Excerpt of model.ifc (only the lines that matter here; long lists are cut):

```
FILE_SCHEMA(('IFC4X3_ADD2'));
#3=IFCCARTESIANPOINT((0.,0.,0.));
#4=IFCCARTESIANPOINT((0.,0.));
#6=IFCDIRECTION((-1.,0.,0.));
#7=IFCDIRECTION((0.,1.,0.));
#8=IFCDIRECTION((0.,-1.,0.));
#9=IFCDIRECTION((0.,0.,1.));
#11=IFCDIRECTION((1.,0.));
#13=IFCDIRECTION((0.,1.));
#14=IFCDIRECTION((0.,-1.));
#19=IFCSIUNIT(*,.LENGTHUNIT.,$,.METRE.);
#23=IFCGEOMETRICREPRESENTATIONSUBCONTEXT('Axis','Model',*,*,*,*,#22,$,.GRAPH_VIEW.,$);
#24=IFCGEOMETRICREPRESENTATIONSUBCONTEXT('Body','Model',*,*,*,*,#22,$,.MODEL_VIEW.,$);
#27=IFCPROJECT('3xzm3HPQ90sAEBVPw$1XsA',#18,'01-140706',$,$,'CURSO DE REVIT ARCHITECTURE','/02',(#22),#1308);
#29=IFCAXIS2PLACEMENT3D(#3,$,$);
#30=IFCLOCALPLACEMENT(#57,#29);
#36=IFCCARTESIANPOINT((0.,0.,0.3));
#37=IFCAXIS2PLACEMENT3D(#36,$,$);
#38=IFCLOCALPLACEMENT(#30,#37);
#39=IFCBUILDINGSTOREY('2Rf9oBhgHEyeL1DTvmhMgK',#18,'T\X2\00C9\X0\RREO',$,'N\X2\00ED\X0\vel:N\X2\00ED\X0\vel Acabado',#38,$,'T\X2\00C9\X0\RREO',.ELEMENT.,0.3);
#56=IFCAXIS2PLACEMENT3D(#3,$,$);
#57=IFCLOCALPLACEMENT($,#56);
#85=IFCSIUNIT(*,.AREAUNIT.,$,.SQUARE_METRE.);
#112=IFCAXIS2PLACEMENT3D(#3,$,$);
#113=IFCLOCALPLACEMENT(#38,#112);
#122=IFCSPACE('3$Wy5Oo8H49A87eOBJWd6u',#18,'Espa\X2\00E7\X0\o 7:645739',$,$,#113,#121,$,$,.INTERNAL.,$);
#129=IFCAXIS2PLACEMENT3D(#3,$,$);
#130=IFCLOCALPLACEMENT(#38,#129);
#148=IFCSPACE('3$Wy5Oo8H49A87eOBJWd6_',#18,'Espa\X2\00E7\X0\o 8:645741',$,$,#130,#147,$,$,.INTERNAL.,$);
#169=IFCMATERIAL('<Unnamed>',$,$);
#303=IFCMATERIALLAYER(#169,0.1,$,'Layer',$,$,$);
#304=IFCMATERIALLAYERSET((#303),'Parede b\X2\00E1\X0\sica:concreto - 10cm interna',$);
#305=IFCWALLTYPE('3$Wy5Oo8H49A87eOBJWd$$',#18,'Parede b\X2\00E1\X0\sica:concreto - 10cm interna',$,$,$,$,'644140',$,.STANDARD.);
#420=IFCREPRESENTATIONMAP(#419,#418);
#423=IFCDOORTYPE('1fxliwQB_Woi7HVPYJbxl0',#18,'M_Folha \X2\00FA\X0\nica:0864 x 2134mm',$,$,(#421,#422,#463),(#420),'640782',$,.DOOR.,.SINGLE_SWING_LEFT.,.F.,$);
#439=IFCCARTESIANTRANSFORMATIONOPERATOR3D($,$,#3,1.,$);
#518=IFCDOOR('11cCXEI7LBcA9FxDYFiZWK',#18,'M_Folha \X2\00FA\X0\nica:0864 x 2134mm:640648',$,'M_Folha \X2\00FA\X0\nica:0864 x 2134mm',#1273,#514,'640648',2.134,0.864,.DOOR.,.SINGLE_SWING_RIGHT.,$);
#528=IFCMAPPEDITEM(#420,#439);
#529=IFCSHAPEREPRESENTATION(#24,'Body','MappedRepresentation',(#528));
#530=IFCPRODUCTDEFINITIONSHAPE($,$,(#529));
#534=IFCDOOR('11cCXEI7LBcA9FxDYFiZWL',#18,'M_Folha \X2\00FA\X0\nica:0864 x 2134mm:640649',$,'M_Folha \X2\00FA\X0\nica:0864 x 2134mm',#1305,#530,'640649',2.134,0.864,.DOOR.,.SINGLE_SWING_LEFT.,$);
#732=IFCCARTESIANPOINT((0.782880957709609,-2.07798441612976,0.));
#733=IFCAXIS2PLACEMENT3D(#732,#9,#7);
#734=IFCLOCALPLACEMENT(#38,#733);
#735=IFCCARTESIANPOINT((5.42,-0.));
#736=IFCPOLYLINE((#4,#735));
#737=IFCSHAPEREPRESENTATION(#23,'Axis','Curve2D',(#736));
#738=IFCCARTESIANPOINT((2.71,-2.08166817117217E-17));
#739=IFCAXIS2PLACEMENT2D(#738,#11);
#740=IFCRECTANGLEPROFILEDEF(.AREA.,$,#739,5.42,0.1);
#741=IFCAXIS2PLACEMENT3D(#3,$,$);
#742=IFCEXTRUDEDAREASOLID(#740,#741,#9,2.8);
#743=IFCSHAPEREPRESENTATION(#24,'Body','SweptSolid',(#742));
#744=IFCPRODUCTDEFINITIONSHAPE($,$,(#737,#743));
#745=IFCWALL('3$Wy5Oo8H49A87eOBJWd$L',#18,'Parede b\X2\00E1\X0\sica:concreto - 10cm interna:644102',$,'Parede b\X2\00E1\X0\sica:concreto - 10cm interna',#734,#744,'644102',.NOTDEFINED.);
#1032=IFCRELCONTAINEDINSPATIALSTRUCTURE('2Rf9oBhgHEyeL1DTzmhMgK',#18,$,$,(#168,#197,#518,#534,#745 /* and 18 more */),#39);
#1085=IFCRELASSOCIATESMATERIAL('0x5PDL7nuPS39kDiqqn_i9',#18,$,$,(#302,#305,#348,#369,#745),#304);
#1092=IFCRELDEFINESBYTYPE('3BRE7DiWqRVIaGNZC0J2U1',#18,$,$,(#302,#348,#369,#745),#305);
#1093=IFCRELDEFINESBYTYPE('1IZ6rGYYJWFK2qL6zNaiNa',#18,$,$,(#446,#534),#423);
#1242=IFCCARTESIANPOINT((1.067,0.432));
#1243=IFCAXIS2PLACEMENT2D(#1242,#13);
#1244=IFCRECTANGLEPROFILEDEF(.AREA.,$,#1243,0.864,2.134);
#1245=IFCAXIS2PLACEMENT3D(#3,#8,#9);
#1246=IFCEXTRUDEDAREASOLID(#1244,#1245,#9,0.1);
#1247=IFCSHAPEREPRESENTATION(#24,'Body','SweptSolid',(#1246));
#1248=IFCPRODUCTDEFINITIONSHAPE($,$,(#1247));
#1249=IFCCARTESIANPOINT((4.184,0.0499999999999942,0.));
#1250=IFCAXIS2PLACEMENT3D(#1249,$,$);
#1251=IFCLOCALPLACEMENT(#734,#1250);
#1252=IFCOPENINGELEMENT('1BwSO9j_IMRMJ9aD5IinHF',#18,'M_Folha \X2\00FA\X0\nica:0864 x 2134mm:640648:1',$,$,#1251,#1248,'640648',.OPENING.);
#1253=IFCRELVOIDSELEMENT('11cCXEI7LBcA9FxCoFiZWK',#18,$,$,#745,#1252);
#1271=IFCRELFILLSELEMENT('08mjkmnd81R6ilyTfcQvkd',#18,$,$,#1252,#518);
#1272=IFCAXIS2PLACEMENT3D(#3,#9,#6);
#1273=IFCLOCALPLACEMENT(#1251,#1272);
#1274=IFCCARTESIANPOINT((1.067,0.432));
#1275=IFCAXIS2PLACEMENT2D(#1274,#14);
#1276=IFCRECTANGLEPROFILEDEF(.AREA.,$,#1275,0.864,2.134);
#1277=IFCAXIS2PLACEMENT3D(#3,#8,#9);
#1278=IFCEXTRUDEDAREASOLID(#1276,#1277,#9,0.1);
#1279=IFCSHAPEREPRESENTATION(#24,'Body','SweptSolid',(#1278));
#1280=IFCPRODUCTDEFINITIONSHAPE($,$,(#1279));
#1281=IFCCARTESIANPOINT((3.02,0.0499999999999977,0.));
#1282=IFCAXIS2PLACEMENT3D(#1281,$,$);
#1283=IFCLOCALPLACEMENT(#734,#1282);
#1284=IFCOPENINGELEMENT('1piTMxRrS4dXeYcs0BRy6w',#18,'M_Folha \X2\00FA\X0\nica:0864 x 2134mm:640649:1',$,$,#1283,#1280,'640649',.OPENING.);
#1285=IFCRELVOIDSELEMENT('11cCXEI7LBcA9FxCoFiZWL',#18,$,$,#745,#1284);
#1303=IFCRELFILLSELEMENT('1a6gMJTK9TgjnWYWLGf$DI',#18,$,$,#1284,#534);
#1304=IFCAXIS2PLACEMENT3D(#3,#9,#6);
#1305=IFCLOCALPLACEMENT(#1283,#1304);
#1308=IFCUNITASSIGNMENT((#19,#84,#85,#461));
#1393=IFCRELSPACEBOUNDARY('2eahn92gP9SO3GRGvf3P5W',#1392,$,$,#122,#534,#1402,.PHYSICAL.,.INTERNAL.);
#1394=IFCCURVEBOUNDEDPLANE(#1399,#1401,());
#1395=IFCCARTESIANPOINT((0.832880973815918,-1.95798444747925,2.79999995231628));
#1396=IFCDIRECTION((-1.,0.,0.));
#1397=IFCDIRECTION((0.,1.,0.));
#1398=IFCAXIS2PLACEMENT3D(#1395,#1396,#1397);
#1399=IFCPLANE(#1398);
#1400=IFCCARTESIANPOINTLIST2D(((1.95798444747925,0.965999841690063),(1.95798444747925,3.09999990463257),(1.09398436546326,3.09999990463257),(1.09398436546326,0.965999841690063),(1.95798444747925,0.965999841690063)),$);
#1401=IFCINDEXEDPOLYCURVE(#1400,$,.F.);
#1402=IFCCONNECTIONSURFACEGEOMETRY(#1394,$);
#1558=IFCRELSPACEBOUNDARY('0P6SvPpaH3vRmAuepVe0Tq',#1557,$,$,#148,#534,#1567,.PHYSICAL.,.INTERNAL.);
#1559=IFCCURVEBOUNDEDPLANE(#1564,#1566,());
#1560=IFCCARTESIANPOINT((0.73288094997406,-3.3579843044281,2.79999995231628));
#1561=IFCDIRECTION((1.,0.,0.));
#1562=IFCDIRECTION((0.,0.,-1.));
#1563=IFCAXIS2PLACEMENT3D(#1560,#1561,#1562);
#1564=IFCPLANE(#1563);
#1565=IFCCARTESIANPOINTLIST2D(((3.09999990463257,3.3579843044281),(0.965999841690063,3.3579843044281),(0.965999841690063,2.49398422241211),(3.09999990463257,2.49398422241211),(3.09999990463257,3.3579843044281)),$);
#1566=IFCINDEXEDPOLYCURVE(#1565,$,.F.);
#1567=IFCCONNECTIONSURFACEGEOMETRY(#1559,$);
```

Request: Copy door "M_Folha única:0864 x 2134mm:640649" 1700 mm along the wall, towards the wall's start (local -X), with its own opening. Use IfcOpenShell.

```python
import numpy as np
import ifcopenshell
import ifcopenshell.api.feature
import ifcopenshell.api.geometry
import ifcopenshell.api.root
import ifcopenshell.geom
import ifcopenshell.util.element
import ifcopenshell.util.placement
import ifcopenshell.util.shape
import ifcopenshell.util.unit

model = ifcopenshell.open("model.ifc")
unit_scale = ifcopenshell.util.unit.calculate_unit_scale(model)
settings = ifcopenshell.geom.settings()


def volume(element):
    """Net volume in cubic metres, openings subtracted."""
    shape = ifcopenshell.geom.create_shape(settings, element)
    return ifcopenshell.util.shape.get_volume(shape.geometry)


def reuse_history(source, copy):
    """copy_class also copies each property set's owner history, people and application; keep the originals."""
    for rel in copy.IsDefinedBy:
        if rel.is_a("IfcRelDefinesByProperties") and (history := rel.RelatingPropertyDefinition.OwnerHistory):
            rel.RelatingPropertyDefinition.OwnerHistory = source.OwnerHistory
            ifcopenshell.util.element.remove_deep2(model, history)


door = model.by_guid("11cCXEI7LBcA9FxDYFiZWL")
opening = door.FillsVoids[0].RelatingOpeningElement
wall = opening.VoidsElements[0].RelatingBuildingElement
before = volume(wall)
shift = ifcopenshell.util.placement.get_local_placement(wall.ObjectPlacement)[:3, 0] * -1.7 / unit_scale

# copy_class copies the void relationship, type, container and properties, but no geometry.
new_opening = ifcopenshell.api.root.copy_class(model, product=opening)
new_opening.Representation = ifcopenshell.util.element.copy_deep(
    model, opening.Representation, exclude=["IfcGeometricRepresentationContext", "IfcRepresentationMap"]
)
new_opening.Name = "M_Folha única:0864 x 2134mm"
new_opening.Tag = None
new_door = ifcopenshell.api.root.copy_class(model, product=door)
new_door.Representation = ifcopenshell.util.element.copy_deep(
    model, door.Representation, exclude=["IfcGeometricRepresentationContext", "IfcRepresentationMap"]
)
new_door.Name = "M_Folha única:0864 x 2134mm"
new_door.Tag = None
reuse_history(door, new_door)
ifcopenshell.api.feature.add_filling(model, opening=new_opening, element=new_door)

for old, new in ((opening, new_opening), (door, new_door)):
    matrix = ifcopenshell.util.placement.get_local_placement(old.ObjectPlacement)
    matrix[:3, 3] += shift
    ifcopenshell.api.geometry.edit_object_placement(model, product=new, matrix=matrix, is_si=False)

# The copied space boundaries still share their surfaces with the original.
for rel in new_door.ProvidesBoundaries:
    if rel.ConnectionGeometry:
        rel.ConnectionGeometry = ifcopenshell.util.element.copy_deep(model, rel.ConnectionGeometry)

# Space boundary surfaces are stored in each space's coordinates; move them too.
for rel in new_door.ProvidesBoundaries:
    if not rel.ConnectionGeometry:
        continue
    surface = rel.ConnectionGeometry.SurfaceOnRelatingElement.BasisSurface
    space_matrix = ifcopenshell.util.placement.get_local_placement(rel.RelatingSpace.ObjectPlacement)
    point = np.array(surface.Position.Location.Coordinates) + space_matrix[:3, :3].T @ shift
    surface.Position = model.createIfcAxis2Placement3D(
        model.createIfcCartesianPoint(point.tolist()), surface.Position.Axis, surface.Position.RefDirection
    )

after = volume(wall)

print(f"wall volume {before:.3f} -> {after:.3f} m3")

model.write("model_edited.ifc")
```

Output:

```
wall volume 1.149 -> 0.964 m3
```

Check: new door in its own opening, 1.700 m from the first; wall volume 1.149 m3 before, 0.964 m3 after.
